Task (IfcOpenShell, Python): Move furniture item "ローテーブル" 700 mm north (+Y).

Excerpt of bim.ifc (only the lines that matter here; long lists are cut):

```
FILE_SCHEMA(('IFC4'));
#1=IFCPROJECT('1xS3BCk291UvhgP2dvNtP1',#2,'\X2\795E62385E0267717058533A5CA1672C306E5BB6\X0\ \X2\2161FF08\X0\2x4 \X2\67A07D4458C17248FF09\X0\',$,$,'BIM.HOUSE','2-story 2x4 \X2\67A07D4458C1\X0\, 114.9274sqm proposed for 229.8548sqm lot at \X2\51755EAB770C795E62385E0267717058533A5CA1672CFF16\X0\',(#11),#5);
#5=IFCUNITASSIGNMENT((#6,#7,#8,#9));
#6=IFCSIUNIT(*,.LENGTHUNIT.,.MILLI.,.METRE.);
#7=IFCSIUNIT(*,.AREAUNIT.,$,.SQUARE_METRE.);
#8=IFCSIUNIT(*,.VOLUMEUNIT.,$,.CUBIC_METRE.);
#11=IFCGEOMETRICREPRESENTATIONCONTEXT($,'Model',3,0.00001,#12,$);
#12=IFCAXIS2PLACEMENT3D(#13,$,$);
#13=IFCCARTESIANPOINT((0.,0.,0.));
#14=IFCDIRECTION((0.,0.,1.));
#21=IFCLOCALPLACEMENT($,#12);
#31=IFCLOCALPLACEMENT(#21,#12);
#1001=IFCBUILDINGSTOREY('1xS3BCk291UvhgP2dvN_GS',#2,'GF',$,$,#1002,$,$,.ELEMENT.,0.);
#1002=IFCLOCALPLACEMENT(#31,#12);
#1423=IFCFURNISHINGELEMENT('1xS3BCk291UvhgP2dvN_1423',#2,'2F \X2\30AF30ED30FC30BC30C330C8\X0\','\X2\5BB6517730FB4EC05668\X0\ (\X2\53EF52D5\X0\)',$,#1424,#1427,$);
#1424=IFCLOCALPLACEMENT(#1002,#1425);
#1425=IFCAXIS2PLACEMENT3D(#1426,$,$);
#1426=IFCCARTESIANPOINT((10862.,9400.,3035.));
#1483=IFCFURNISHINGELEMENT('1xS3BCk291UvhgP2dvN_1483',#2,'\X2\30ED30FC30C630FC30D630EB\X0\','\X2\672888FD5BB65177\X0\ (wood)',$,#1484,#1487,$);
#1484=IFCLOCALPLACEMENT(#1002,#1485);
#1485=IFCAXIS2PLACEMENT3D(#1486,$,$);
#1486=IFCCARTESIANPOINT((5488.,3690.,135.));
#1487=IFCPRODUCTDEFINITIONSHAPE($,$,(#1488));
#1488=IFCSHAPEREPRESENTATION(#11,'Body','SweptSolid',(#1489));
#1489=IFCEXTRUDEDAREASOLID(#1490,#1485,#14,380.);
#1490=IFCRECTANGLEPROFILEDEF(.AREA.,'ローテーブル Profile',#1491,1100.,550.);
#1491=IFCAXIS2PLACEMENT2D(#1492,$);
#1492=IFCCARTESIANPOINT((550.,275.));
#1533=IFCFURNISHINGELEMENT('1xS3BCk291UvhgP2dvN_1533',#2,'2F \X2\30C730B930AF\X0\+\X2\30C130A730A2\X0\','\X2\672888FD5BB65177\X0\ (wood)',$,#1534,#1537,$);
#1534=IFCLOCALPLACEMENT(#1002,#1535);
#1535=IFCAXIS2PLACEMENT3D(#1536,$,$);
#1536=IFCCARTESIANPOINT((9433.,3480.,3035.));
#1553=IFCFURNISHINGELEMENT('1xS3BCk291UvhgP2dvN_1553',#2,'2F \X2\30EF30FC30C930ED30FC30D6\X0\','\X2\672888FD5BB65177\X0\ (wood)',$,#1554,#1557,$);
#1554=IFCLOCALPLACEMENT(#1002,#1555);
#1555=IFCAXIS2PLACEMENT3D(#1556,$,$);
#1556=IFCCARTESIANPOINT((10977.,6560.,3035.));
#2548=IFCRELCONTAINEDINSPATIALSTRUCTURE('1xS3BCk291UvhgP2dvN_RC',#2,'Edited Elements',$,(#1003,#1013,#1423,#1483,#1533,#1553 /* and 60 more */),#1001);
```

```python
import ifcopenshell
import ifcopenshell.api.geometry
import ifcopenshell.util.placement
import ifcopenshell.util.unit

model = ifcopenshell.open("bim.ifc")
unit_scale = ifcopenshell.util.unit.calculate_unit_scale(model)

item = model.by_guid("1xS3BCk291UvhgP2dvN_1483")
matrix = ifcopenshell.util.placement.get_local_placement(item.ObjectPlacement)
matrix[1, 3] += 0.7 / unit_scale
ifcopenshell.api.geometry.edit_object_placement(model, product=item, matrix=matrix, is_si=False)

print(ifcopenshell.util.placement.get_local_placement(item.ObjectPlacement).round(3) + 0.0)

model.write("bim_rev.ifc")
```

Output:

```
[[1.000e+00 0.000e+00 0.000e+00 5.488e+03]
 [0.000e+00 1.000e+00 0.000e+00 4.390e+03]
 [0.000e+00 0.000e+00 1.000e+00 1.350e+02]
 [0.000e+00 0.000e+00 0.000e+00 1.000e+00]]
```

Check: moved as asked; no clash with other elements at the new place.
